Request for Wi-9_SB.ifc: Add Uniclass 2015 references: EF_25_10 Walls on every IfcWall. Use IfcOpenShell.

First a look at what the model holds.

```python
import ifcopenshell

model = ifcopenshell.open("Wi-9_SB.ifc")
print(model.schema)
print("classifications:", [c.Name for c in model.by_type("IfcClassification")])
for ifc_class in ("IfcDoor", "IfcRoof", "IfcStair", "IfcWall", "IfcWindow"):
    print(ifc_class, len(model.by_type(ifc_class)))
```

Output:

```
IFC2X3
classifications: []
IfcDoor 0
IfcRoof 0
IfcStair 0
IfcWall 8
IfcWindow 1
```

```python
import ifcopenshell
import ifcopenshell.api.classification

model = ifcopenshell.open("Wi-9_SB.ifc")

# IFC2X3 requires Source and Edition and has no link from the project to the system.
system = model.create_entity("IfcClassification", Source="NBS", Edition="2015", Name="Uniclass 2015")

codes = {
    "IfcWall": ("EF_25_10", "Walls"),
}
for ifc_class, (code, name) in codes.items():
    products = model.by_type(ifc_class)
    ifcopenshell.api.classification.add_reference(
        model, products=products, classification=system, identification=code, name=name
    )
    print(code, len(products))

model.write("Wi-9_SB_rev.ifc")
```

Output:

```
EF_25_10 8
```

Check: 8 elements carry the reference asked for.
